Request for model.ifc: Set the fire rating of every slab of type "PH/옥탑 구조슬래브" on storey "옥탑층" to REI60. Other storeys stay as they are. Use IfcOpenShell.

First a look at what the model holds.

```python
import ifcopenshell
import ifcopenshell.util.element

model = ifcopenshell.open("model.ifc")
print(model.schema)
storey = next(s for s in model.by_type("IfcBuildingStorey") if s.Name == "옥탑층")
slabs = [e for e in ifcopenshell.util.element.get_decomposition(storey) if e.is_a("IfcSlab")]
seen = {}
for e in slabs:
    element_type = ifcopenshell.util.element.get_type(e)
    key = (element_type.Name if element_type != e and element_type else None, ifcopenshell.util.element.get_pset(e, "Pset_SlabCommon", "FireRating"))
    seen[key] = seen.get(key, 0) + 1
for (name, value), count in sorted(seen.items(), key=str):
    print(count, "x", name, "|", value)
```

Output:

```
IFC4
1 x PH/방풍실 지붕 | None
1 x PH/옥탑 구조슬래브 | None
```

```python
import ifcopenshell
import ifcopenshell.api.pset
import ifcopenshell.util.element

model = ifcopenshell.open("model.ifc")

storey = next(s for s in model.by_type("IfcBuildingStorey") if s.Name == "옥탑층")
slabs = [e for e in ifcopenshell.util.element.get_decomposition(storey) if e.is_a("IfcSlab")]

count = 0
for e in slabs:
    element_type = ifcopenshell.util.element.get_type(e)
    if element_type in (None, e) or element_type.Name != "PH/옥탑 구조슬래브":
        continue
    # add_pset returns the element's existing set when there is one.
    pset = ifcopenshell.api.pset.add_pset(model, product=e, name="Pset_SlabCommon")
    ifcopenshell.api.pset.edit_pset(model, pset=pset, properties={"FireRating": "REI60"})
    count += 1

print(count, "slabs updated")

model.write("model_rev.ifc")
```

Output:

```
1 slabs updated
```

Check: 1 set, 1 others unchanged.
